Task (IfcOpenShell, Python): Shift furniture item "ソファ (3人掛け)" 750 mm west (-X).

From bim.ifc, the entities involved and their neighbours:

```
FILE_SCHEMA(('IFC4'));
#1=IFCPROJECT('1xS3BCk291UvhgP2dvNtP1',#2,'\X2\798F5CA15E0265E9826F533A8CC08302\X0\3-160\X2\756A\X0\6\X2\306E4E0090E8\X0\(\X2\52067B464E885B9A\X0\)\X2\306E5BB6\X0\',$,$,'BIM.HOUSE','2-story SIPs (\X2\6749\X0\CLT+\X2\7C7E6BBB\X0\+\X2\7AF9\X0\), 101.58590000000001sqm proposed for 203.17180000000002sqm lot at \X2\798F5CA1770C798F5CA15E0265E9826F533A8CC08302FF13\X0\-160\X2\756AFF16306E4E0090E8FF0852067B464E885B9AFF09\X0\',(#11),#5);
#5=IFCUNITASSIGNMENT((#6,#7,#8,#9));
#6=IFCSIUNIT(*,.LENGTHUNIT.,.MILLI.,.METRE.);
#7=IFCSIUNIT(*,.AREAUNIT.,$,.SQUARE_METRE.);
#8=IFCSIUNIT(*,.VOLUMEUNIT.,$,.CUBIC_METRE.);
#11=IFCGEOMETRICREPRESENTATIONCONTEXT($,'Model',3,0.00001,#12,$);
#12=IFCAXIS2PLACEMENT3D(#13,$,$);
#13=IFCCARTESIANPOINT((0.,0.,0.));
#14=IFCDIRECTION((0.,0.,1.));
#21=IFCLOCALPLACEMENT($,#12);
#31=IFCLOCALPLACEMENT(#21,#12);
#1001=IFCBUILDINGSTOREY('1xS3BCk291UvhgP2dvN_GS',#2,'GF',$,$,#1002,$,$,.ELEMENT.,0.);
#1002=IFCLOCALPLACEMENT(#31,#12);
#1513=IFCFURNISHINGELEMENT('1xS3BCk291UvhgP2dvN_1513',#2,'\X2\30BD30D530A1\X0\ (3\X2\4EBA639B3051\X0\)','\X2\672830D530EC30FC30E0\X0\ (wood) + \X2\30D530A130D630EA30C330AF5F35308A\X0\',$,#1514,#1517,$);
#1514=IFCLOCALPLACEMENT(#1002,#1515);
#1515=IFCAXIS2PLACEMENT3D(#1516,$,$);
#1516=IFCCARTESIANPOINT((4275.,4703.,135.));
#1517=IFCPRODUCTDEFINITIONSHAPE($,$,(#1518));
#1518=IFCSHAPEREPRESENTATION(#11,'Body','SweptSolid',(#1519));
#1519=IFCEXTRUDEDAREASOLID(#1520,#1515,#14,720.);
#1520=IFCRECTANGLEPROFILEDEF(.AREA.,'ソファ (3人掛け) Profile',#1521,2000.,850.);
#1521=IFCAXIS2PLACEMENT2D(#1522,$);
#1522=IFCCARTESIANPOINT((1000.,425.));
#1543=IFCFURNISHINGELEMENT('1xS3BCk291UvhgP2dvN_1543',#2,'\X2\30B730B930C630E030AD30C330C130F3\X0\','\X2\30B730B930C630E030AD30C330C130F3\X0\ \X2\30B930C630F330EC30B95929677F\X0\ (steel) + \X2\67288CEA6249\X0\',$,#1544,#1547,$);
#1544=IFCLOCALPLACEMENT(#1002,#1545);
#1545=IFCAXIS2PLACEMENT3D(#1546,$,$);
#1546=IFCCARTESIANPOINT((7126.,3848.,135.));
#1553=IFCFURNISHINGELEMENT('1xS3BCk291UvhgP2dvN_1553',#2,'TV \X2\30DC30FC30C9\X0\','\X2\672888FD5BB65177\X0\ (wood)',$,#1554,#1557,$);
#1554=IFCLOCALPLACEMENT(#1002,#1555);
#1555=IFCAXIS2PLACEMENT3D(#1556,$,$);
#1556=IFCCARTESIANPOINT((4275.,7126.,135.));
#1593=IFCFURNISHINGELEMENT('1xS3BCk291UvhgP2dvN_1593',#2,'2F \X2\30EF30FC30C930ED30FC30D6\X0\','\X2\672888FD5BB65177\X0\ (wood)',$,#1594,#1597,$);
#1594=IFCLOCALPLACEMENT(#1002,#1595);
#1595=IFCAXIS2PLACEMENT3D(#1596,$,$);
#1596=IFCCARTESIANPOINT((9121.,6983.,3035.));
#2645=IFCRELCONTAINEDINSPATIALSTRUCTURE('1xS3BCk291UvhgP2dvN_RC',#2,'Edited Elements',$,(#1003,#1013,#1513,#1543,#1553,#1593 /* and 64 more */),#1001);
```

```python
import ifcopenshell
import ifcopenshell.api.geometry
import ifcopenshell.util.placement

model = ifcopenshell.open("bim.ifc")

item = model.by_guid("1xS3BCk291UvhgP2dvN_1513")
matrix = ifcopenshell.util.placement.get_local_placement(item.ObjectPlacement)
matrix[0, 3] -= 750.0
ifcopenshell.api.geometry.edit_object_placement(model, product=item, matrix=matrix, is_si=False)

print(ifcopenshell.util.placement.get_local_placement(item.ObjectPlacement).round(3) + 0.0)

model.write("bim_updated.ifc")
```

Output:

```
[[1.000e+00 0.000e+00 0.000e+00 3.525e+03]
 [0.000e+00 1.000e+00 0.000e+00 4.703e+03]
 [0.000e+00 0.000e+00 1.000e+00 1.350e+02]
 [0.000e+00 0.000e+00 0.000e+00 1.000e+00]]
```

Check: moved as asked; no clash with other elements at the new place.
